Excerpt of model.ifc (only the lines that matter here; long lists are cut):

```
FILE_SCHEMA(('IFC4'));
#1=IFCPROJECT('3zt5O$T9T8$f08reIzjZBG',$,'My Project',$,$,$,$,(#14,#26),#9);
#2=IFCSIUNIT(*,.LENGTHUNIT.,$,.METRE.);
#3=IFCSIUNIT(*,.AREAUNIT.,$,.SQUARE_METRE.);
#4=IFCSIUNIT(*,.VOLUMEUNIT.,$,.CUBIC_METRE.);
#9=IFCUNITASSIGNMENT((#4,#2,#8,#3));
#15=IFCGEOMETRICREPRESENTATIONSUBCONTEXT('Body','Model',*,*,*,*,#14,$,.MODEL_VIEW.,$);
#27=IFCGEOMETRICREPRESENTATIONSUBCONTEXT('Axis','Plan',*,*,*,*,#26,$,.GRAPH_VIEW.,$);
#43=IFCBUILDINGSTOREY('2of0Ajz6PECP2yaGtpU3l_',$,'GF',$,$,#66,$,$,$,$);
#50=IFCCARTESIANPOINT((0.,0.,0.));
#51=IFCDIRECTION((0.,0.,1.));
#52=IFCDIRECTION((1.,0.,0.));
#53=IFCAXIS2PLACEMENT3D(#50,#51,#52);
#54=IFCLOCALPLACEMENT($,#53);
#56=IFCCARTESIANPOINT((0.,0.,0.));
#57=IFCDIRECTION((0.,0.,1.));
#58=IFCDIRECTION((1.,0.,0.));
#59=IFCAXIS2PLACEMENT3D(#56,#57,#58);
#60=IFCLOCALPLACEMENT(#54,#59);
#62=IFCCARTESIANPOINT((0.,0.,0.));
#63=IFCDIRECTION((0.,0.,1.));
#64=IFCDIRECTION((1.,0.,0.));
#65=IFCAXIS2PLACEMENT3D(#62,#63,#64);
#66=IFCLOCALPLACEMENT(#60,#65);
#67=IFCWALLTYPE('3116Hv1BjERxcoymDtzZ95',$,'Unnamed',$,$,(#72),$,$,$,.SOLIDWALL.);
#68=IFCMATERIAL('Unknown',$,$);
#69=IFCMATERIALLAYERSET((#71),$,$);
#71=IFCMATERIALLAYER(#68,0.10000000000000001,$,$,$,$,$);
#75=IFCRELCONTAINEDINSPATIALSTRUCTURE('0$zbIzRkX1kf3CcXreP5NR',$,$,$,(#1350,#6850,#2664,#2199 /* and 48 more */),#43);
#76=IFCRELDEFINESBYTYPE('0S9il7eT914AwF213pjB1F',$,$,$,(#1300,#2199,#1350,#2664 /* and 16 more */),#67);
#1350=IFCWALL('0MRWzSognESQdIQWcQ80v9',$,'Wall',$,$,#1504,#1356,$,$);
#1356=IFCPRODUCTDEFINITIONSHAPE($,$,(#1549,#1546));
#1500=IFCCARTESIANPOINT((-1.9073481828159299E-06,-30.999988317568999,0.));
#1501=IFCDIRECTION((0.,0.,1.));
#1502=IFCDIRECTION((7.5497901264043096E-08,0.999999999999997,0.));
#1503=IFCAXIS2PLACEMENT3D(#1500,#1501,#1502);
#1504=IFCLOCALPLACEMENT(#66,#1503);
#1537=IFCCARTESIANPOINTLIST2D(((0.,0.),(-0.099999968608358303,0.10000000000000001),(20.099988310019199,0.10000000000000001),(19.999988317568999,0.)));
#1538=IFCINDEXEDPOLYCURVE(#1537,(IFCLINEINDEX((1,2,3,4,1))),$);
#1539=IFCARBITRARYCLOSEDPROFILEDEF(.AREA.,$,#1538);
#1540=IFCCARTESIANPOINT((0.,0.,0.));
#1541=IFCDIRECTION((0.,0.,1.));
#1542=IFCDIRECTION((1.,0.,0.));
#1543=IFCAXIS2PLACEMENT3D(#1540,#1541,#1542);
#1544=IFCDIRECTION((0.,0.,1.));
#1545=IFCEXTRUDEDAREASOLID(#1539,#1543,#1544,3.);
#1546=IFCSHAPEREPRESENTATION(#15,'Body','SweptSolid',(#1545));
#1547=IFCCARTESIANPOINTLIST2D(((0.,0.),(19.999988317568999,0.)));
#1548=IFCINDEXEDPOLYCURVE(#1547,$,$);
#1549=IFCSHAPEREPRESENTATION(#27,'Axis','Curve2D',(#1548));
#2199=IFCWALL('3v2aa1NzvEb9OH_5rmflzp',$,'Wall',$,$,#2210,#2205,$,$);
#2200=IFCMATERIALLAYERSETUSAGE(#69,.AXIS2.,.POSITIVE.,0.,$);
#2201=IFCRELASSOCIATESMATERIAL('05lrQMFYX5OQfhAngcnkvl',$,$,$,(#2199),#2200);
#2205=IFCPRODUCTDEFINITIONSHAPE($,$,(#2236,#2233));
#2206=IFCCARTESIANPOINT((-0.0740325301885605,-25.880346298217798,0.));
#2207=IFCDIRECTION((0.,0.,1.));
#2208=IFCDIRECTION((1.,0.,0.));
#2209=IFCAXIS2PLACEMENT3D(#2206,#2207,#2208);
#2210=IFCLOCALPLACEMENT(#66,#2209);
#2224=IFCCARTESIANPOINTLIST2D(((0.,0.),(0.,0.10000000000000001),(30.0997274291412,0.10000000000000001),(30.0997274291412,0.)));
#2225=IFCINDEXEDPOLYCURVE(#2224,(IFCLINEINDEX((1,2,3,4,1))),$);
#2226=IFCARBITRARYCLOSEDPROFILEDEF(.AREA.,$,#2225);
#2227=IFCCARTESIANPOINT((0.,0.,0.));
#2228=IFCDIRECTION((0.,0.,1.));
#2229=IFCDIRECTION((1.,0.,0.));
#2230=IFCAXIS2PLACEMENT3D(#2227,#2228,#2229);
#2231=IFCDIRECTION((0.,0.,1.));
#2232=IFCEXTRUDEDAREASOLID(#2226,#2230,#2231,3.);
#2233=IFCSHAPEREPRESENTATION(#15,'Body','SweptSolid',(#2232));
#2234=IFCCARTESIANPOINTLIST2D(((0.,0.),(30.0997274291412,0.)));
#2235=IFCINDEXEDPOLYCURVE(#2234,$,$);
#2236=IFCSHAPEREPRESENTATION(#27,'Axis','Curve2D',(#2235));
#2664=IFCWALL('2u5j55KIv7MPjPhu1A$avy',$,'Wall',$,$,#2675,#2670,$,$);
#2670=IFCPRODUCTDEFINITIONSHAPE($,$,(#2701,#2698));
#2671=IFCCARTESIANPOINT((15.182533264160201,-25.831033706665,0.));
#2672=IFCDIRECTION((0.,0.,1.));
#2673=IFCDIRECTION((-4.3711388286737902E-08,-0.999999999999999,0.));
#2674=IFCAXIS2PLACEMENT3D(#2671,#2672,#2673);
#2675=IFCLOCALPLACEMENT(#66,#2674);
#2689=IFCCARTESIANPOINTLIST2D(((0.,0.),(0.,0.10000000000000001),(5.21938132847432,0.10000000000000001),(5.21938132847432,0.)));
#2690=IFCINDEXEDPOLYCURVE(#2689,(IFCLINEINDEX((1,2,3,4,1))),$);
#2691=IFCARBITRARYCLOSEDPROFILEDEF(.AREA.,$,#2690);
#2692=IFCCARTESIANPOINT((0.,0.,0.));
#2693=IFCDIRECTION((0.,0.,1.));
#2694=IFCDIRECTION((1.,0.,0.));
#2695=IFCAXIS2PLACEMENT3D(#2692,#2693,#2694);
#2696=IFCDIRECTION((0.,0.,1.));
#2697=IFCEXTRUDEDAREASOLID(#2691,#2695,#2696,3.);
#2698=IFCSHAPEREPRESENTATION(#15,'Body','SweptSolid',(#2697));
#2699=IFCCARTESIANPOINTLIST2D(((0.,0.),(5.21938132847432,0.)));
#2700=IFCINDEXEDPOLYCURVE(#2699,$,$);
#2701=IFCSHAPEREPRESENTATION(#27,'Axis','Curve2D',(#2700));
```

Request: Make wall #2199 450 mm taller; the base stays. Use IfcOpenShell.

```python
import ifcopenshell
import ifcopenshell.geom
import ifcopenshell.util.representation
import ifcopenshell.util.shape
import ifcopenshell.util.unit

model = ifcopenshell.open("model.ifc")
unit_scale = ifcopenshell.util.unit.calculate_unit_scale(model)
settings = ifcopenshell.geom.settings()


def volume(element):
    """Net volume in cubic metres, openings subtracted."""
    shape = ifcopenshell.geom.create_shape(settings, element)
    return ifcopenshell.util.shape.get_volume(shape.geometry)


wall = model.by_guid("3v2aa1NzvEb9OH_5rmflzp")
before = volume(wall)

body = ifcopenshell.util.representation.get_representation(wall, "Model", "Body")
solid = body.Items[0]
old_height = solid.Depth
solid.Depth += 0.45 / unit_scale
after = volume(wall)

print(f"height {old_height:g} -> {solid.Depth:g}, volume {before:.3f} -> {after:.3f} m3")

model.write("model_edited.ifc")
```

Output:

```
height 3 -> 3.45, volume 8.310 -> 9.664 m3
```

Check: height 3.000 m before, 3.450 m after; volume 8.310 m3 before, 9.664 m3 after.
